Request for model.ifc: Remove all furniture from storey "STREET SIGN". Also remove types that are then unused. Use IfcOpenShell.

First a look at what the model holds.

```python
import ifcopenshell
import ifcopenshell.util.element

model = ifcopenshell.open("model.ifc")
print(model.schema)
storey = next(s for s in model.by_type("IfcBuildingStorey") if s.Name == "STREET SIGN")
furniture = [e for e in ifcopenshell.util.element.get_decomposition(storey) if e.is_a("IfcFurnishingElement")]
seen = {}
for e in furniture:
    element_type = ifcopenshell.util.element.get_type(e)
    name = element_type.Name if element_type not in (None, e) else None
    seen[name] = seen.get(name, 0) + 1
for name, count in sorted(seen.items(), key=str):
    print(count, "x", name)
```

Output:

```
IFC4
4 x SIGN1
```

```python
import ifcopenshell
import ifcopenshell.api.root
import ifcopenshell.util.element

model = ifcopenshell.open("model.ifc")

storey = next(s for s in model.by_type("IfcBuildingStorey") if s.Name == "STREET SIGN")
furniture = [e for e in ifcopenshell.util.element.get_decomposition(storey) if e.is_a("IfcFurnishingElement")]
types = {ifcopenshell.util.element.get_type(e) for e in furniture} - {None, *furniture}

for e in furniture:
    ifcopenshell.api.root.remove_product(model, product=e)
print(len(furniture), "removed")

unused = [t for t in types if not ifcopenshell.util.element.get_types(t)]
for t in unused:
    ifcopenshell.api.root.remove_product(model, product=t)
print(len(unused), "unused types removed")

model.write("model_edited.ifc")
```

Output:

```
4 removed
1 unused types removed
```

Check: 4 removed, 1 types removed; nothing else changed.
